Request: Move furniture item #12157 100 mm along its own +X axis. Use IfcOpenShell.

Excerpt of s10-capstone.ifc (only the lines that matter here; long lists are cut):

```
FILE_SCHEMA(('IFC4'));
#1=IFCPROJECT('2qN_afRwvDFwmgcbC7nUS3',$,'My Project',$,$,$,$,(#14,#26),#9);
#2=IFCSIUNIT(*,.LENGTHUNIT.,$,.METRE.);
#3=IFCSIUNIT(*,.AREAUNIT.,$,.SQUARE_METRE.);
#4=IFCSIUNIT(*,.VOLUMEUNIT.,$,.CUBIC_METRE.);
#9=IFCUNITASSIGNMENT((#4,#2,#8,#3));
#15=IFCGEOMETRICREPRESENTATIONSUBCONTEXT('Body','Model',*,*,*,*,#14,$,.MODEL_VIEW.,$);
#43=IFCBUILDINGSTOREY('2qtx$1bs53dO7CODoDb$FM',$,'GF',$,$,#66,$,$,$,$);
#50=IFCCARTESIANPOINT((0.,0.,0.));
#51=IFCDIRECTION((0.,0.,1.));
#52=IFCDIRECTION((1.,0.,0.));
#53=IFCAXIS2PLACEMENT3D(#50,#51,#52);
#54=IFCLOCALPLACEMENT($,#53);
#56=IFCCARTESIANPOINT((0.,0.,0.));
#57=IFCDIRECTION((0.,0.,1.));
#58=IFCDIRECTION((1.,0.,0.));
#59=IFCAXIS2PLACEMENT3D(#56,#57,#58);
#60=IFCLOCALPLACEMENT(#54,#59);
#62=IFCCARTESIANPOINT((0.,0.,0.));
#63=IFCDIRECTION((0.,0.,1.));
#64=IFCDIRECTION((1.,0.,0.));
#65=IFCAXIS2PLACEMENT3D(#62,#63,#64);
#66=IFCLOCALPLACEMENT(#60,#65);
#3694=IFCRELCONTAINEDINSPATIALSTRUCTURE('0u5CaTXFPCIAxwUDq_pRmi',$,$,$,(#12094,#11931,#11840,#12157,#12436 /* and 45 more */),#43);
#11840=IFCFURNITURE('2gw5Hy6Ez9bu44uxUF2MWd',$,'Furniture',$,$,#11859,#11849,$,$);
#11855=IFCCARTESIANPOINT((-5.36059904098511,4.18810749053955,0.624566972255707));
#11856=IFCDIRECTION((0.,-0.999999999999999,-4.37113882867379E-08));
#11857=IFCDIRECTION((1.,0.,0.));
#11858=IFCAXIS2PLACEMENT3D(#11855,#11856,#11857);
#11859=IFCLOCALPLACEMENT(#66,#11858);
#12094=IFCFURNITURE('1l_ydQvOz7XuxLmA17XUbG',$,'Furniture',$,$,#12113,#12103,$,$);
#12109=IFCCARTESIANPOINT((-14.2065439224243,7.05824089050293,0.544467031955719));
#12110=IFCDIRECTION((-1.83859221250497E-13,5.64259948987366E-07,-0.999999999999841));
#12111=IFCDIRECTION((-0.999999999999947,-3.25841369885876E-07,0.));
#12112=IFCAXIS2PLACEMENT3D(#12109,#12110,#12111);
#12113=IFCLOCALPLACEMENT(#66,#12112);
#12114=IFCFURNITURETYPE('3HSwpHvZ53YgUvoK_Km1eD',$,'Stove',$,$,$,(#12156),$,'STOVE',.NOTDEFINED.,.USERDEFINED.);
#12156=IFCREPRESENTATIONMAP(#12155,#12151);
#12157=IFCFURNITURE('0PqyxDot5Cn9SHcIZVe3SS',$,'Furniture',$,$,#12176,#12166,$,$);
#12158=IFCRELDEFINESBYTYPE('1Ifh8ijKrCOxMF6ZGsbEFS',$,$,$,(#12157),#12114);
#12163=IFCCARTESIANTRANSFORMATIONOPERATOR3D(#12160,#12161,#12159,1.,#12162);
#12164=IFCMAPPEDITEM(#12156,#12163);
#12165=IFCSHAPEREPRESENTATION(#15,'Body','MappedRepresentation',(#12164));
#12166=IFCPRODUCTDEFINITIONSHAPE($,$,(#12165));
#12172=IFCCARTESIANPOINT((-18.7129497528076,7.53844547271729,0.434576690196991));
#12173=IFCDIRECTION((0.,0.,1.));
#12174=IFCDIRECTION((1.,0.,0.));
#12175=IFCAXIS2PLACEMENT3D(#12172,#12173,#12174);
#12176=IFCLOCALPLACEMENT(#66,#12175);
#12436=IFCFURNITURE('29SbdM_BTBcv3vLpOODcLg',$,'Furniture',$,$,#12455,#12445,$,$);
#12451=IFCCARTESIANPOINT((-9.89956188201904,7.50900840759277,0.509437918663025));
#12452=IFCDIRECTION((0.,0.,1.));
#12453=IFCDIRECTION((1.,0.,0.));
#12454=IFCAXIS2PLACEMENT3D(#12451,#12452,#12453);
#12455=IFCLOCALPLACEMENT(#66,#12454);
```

```python
import ifcopenshell
import ifcopenshell.api.geometry
import ifcopenshell.util.placement

model = ifcopenshell.open("s10-capstone.ifc")

item = model.by_id(12157)
matrix = ifcopenshell.util.placement.get_local_placement(item.ObjectPlacement)
matrix[:3, 3] += matrix[:3, 0] * 0.1
ifcopenshell.api.geometry.edit_object_placement(model, product=item, matrix=matrix, is_si=False)

print(ifcopenshell.util.placement.get_local_placement(item.ObjectPlacement).round(3) + 0.0)

model.write("s10-capstone_edited.ifc")
```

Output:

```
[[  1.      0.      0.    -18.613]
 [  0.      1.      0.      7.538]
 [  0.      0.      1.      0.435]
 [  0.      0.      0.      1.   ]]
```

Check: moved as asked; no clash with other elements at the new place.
